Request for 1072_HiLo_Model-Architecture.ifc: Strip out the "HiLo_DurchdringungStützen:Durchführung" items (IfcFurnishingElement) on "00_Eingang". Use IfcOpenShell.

First a look at what the model holds.

```python
import ifcopenshell
import ifcopenshell.util.element

model = ifcopenshell.open("1072_HiLo_Model-Architecture.ifc")
print(model.schema)
storey = next(s for s in model.by_type("IfcBuildingStorey") if s.Name == "00_Eingang")
furniture = [e for e in ifcopenshell.util.element.get_decomposition(storey) if e.is_a("IfcFurnishingElement")]
seen = {}
for e in furniture:
    element_type = ifcopenshell.util.element.get_type(e)
    name = element_type.Name if element_type not in (None, e) else None
    seen[name] = seen.get(name, 0) + 1
for name, count in sorted(seen.items(), key=str):
    print(count, "x", name)
```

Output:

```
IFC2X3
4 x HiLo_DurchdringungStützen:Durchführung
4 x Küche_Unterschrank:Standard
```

```python
import ifcopenshell
import ifcopenshell.api.root
import ifcopenshell.util.element

model = ifcopenshell.open("1072_HiLo_Model-Architecture.ifc")

storey = next(s for s in model.by_type("IfcBuildingStorey") if s.Name == "00_Eingang")
furniture = [e for e in ifcopenshell.util.element.get_decomposition(storey) if e.is_a("IfcFurnishingElement")]
targets = [e for e in furniture if (t := ifcopenshell.util.element.get_type(e)) not in (None, e) and t.Name == "HiLo_DurchdringungStützen:Durchführung"]

for e in targets:
    ifcopenshell.api.root.remove_product(model, product=e)
print(len(targets), "removed")

model.write("1072_HiLo_Model-Architecture_updated.ifc")
```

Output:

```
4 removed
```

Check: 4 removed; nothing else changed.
